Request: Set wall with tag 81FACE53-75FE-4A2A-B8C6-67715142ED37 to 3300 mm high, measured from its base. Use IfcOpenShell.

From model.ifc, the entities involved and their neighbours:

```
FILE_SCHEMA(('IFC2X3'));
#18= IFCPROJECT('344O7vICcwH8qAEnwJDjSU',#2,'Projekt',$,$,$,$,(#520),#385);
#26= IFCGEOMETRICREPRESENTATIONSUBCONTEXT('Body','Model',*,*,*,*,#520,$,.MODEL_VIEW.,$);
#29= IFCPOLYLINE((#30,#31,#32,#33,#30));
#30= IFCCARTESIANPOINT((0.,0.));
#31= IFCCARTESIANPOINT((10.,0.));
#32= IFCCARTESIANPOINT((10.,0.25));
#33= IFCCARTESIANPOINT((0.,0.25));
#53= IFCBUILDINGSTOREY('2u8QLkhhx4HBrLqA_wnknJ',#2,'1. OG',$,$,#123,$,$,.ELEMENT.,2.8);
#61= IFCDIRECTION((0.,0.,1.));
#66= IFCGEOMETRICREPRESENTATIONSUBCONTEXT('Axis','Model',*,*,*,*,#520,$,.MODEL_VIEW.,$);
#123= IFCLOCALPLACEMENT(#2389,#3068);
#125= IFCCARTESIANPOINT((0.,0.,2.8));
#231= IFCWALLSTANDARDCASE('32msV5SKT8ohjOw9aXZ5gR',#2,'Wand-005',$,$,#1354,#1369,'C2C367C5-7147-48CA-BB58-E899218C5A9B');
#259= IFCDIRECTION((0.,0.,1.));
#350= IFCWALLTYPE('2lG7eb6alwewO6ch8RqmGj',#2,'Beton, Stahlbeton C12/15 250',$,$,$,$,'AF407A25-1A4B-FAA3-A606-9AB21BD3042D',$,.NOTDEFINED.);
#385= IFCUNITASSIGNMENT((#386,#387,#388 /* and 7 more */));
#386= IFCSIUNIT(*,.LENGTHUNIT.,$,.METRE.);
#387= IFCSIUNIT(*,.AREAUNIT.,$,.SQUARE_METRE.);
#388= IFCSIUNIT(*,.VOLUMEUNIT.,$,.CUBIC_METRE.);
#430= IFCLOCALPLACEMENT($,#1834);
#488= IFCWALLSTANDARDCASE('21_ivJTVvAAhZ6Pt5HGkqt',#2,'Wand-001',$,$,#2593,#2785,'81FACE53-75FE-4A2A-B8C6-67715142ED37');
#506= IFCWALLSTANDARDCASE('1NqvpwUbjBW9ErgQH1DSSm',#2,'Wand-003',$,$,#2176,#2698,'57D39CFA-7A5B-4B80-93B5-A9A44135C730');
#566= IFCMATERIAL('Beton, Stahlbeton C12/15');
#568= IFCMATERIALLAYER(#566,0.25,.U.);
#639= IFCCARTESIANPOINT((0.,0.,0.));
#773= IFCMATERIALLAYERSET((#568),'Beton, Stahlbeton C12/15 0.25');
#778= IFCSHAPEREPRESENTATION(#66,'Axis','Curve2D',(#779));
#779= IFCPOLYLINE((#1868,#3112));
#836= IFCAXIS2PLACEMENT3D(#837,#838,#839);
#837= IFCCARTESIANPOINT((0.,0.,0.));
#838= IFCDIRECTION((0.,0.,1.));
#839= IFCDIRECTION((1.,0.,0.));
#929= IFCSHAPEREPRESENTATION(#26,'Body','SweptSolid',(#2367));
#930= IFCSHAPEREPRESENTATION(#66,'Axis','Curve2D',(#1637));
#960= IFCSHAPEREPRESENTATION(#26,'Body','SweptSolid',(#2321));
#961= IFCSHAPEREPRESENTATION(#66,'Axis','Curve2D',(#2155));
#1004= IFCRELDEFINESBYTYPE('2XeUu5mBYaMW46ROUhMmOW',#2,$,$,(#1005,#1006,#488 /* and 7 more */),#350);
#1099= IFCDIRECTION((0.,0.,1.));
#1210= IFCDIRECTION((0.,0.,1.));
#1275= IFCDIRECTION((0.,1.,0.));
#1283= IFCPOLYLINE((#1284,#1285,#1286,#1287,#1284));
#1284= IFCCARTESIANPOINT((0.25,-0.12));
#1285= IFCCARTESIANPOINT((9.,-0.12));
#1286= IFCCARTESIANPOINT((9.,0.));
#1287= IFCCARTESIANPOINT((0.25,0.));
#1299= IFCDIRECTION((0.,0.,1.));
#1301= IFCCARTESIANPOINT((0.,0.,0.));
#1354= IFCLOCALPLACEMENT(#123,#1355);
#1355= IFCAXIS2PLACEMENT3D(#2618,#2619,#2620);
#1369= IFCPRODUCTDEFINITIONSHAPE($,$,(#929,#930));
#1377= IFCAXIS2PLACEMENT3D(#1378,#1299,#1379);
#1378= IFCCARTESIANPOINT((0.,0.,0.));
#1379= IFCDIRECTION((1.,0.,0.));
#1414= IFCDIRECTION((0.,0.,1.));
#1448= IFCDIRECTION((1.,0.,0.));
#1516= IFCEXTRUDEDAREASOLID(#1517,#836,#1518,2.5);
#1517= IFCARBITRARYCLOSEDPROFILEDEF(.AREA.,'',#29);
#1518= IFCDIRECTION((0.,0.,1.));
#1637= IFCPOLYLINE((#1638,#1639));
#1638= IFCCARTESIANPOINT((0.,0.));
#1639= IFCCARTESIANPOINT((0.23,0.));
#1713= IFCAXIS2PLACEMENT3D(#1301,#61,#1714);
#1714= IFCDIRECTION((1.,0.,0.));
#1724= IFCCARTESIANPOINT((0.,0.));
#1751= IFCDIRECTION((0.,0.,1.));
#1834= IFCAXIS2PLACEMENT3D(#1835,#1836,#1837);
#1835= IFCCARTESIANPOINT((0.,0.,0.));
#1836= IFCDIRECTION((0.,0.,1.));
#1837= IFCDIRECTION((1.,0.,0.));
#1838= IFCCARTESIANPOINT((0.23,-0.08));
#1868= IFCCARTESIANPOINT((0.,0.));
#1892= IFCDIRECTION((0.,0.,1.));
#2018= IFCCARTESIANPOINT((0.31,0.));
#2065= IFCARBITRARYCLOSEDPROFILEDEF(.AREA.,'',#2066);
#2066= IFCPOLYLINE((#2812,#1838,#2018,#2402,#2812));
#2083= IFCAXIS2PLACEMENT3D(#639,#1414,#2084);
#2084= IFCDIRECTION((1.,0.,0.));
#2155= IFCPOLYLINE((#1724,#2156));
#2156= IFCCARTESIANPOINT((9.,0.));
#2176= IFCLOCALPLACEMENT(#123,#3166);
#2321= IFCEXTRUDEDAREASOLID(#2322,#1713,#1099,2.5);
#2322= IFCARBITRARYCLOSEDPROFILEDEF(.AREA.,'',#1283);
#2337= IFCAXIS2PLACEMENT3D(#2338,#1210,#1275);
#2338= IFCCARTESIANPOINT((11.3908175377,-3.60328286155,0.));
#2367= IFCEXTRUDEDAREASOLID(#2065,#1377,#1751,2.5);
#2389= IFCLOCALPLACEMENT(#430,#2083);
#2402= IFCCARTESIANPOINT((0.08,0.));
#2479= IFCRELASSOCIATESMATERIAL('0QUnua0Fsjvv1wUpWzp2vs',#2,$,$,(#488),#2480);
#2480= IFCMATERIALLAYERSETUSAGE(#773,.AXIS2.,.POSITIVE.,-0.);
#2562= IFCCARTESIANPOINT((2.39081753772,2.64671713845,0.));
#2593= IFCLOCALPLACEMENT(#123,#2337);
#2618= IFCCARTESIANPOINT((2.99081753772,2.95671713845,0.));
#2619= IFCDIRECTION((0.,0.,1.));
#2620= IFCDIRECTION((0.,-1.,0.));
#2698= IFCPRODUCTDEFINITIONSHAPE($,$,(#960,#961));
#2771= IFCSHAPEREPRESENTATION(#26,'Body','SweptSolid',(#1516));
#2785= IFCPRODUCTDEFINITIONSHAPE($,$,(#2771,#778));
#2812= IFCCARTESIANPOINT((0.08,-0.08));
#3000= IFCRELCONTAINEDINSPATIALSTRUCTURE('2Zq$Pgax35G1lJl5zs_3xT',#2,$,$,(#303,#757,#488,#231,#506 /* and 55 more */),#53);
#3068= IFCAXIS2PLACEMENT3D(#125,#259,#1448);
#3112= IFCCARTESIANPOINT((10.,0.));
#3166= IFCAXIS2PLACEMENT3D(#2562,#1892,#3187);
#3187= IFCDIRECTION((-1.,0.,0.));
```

```python
import ifcopenshell
import ifcopenshell.geom
import ifcopenshell.util.representation
import ifcopenshell.util.shape
import ifcopenshell.util.unit

model = ifcopenshell.open("model.ifc")
unit_scale = ifcopenshell.util.unit.calculate_unit_scale(model)
settings = ifcopenshell.geom.settings()


def volume(element):
    """Net volume in cubic metres, openings subtracted."""
    shape = ifcopenshell.geom.create_shape(settings, element)
    return ifcopenshell.util.shape.get_volume(shape.geometry)


wall = model.by_guid("21_ivJTVvAAhZ6Pt5HGkqt")
before = volume(wall)

body = ifcopenshell.util.representation.get_representation(wall, "Model", "Body")
solid = body.Items[0]
old_height = solid.Depth
solid.Depth = 3.3 / unit_scale
after = volume(wall)

print(f"height {old_height:g} -> {solid.Depth:g}, volume {before:.3f} -> {after:.3f} m3")

model.write("model-out.ifc")
```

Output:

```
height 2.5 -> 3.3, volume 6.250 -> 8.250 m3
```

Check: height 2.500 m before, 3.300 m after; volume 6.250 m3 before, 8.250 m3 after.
